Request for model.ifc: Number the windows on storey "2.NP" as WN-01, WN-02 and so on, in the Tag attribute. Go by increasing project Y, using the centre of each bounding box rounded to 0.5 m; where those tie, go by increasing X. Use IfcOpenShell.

First a look at what the model holds.

```python
import ifcopenshell
import ifcopenshell.util.element
import ifcopenshell.util.placement

model = ifcopenshell.open("model.ifc")
print(model.schema)
storey = next(s for s in model.by_type("IfcBuildingStorey") if s.Name == "2.NP")
windows = [e for e in ifcopenshell.util.element.get_decomposition(storey) if e.is_a("IfcWindow")]
for e in sorted(windows, key=lambda e: e.id()):
    origin = ifcopenshell.util.placement.get_local_placement(e.ObjectPlacement)[:3, 3]
    print(e.id(), e.Tag, e.Name, origin.round(2) + 0.0, sep=" | ")
```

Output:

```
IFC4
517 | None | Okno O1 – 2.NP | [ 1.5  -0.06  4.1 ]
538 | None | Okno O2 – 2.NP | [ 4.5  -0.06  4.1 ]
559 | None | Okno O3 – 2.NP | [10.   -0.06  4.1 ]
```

```python
import ifcopenshell
import ifcopenshell.geom
import ifcopenshell.util.element
import ifcopenshell.util.shape

model = ifcopenshell.open("model.ifc")
settings = ifcopenshell.geom.settings()
settings.set("use-world-coords", True)


def centre(element):
    shape = ifcopenshell.geom.create_shape(settings, element)
    return ifcopenshell.util.shape.get_bbox_centroid(shape.geometry)


storey = next(s for s in model.by_type("IfcBuildingStorey") if s.Name == "2.NP")
windows = [e for e in ifcopenshell.util.element.get_decomposition(storey) if e.is_a("IfcWindow")]

# Insertion points can sit at a corner or the storey origin, so sort by the geometry (in metres).
centres = {e: centre(e) for e in windows}
windows.sort(key=lambda e: (round(centres[e][1] / 0.5), centres[e][0]))

for i, e in enumerate(windows, start=1):
    number = f"WN-{i:02d}"
    e.Tag = number
    print(e.id(), number)

model.write("model_edited.ifc")
```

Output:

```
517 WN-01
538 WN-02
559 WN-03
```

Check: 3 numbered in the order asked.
